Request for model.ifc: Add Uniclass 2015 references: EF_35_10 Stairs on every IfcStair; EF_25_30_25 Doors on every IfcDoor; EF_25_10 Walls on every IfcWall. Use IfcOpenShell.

First a look at what the model holds.

```python
import ifcopenshell

model = ifcopenshell.open("model.ifc")
print(model.schema)
print("classifications:", [c.Name for c in model.by_type("IfcClassification")])
for ifc_class in ("IfcDoor", "IfcRoof", "IfcStair", "IfcWall", "IfcWindow"):
    print(ifc_class, len(model.by_type(ifc_class)))
```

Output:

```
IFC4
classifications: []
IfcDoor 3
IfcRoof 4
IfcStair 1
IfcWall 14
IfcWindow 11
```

```python
import ifcopenshell
import ifcopenshell.api.classification

model = ifcopenshell.open("model.ifc")

system = ifcopenshell.api.classification.add_classification(model, classification="Uniclass 2015")

codes = {
    "IfcStair": ("EF_35_10", "Stairs"),
    "IfcDoor": ("EF_25_30_25", "Doors"),
    "IfcWall": ("EF_25_10", "Walls"),
}
for ifc_class, (code, name) in codes.items():
    products = model.by_type(ifc_class)
    ifcopenshell.api.classification.add_reference(
        model, products=products, classification=system, identification=code, name=name
    )
    print(code, len(products))

model.write("model_updated.ifc")
```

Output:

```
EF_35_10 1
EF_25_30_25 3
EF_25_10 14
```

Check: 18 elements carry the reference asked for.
